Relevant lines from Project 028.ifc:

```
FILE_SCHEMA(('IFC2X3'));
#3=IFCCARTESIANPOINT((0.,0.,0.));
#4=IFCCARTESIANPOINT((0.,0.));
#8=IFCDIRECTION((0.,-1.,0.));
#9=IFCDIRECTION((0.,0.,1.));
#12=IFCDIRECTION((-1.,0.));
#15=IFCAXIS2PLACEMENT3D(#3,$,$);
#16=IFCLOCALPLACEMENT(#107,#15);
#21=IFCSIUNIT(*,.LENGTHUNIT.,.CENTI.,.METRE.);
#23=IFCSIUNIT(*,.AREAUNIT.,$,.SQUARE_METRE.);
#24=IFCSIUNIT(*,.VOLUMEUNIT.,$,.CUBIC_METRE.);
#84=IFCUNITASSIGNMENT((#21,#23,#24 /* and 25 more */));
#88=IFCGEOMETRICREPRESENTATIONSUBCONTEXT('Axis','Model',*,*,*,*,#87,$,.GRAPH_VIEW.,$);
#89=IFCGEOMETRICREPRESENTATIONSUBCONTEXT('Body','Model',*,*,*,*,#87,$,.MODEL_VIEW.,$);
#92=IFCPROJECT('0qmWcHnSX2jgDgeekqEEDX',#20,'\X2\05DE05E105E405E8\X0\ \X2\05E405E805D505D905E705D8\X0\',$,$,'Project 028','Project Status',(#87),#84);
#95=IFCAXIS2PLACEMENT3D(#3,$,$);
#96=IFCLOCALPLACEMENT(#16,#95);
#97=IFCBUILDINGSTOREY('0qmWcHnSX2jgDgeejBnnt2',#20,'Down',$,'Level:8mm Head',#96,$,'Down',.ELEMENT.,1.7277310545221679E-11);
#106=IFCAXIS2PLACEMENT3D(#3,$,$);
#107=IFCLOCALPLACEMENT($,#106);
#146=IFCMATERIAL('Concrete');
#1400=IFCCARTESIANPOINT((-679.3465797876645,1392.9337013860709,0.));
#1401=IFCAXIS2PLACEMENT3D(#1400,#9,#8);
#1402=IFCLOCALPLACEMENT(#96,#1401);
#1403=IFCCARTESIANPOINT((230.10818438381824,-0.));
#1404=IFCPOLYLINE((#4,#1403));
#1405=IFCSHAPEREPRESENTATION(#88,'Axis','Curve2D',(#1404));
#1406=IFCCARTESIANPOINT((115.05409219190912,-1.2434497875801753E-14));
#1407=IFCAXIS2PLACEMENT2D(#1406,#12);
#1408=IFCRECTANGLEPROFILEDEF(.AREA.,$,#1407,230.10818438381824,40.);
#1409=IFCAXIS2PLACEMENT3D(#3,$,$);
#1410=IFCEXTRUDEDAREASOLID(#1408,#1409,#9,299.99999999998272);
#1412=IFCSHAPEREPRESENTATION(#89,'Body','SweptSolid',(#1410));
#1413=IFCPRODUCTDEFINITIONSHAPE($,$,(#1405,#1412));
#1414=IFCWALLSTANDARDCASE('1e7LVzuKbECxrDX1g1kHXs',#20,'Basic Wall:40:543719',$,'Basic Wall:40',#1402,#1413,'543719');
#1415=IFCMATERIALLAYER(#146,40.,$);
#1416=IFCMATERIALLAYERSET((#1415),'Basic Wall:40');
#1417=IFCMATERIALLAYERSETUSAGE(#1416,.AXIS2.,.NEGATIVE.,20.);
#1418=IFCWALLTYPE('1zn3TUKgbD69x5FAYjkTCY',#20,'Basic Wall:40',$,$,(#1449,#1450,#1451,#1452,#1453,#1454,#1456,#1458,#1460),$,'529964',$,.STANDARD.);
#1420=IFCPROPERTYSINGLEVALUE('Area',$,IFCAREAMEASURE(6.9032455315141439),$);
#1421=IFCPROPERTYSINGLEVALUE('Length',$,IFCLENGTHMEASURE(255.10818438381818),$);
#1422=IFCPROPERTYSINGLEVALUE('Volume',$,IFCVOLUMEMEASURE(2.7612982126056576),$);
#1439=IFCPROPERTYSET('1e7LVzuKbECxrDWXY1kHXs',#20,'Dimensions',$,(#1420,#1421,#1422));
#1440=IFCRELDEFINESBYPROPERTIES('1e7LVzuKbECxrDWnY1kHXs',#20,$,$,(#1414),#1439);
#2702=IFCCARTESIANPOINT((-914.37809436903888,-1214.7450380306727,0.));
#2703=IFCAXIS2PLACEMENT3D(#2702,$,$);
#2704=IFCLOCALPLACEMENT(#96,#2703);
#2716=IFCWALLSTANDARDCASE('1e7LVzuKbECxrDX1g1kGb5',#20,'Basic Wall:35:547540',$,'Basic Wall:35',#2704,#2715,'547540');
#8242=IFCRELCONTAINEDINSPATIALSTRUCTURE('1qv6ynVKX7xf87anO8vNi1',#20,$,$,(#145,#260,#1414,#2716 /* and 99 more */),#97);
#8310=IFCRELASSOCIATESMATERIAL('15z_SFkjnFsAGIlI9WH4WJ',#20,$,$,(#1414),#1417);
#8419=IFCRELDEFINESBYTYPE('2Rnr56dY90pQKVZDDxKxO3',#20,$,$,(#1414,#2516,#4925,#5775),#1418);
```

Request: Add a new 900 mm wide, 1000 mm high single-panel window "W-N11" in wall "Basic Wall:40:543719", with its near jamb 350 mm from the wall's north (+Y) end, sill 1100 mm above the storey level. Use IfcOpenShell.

```python
import numpy as np
import ifcopenshell
import ifcopenshell.api.feature
import ifcopenshell.api.geometry
import ifcopenshell.api.pset
import ifcopenshell.api.root
import ifcopenshell.api.spatial
import ifcopenshell.api.type
import ifcopenshell.geom
import ifcopenshell.util.element
import ifcopenshell.util.placement
import ifcopenshell.util.representation
import ifcopenshell.util.shape
import ifcopenshell.util.unit

model = ifcopenshell.open("Project 028.ifc")
unit_scale = ifcopenshell.util.unit.calculate_unit_scale(model)
area_scale = ifcopenshell.util.unit.calculate_unit_scale(model, "AREAUNIT")
volume_scale = ifcopenshell.util.unit.calculate_unit_scale(model, "VOLUMEUNIT")
settings = ifcopenshell.geom.settings()


def volume(element):
    """Net volume in cubic metres, openings subtracted."""
    shape = ifcopenshell.geom.create_shape(settings, element)
    return ifcopenshell.util.shape.get_volume(shape.geometry)


wall = model.by_id(1414)
storey = ifcopenshell.util.element.get_container(wall, ifc_class="IfcBuildingStorey")
context = ifcopenshell.util.representation.get_context(model, "Model", "Body", "MODEL_VIEW")
before = volume(wall)

width, height, from_end, sill = 0.9, 1, 0.35, 1.1  # metres

# The wall runs along its own X axis, and the end named is its -X end.
wall_shape = ifcopenshell.geom.create_shape(settings, wall)
x, y, z = ifcopenshell.util.shape.get_vertices(wall_shape.geometry).T
start = x.min() + from_end
face, thickness = float(y.min()), float(y.max() - y.min())
wall_matrix = ifcopenshell.util.placement.get_local_placement(wall.ObjectPlacement)
level = ifcopenshell.util.placement.get_local_placement(storey.ObjectPlacement)[2, 3]


def in_wall(x, y):
    """Placement at x, y metres in the wall's axes, at sill height."""
    matrix = wall_matrix.copy()
    matrix[:, 3] = wall_matrix @ np.array([x / unit_scale, y / unit_scale, 0.0, 1.0])
    matrix[2, 3] = level + sill / unit_scale
    return matrix


# Opening: a box that overshoots both wall faces by 50 mm.
opening = ifcopenshell.api.root.create_entity(model, ifc_class="IfcOpeningElement")
box = ifcopenshell.api.geometry.add_wall_representation(
    model, context=context, length=width, height=height, thickness=thickness + 0.1
)
ifcopenshell.api.geometry.assign_representation(model, product=opening, representation=box)
ifcopenshell.api.geometry.edit_object_placement(model, product=opening, matrix=in_wall(start, face - 0.05), is_si=False)
ifcopenshell.api.feature.add_feature(model, feature=opening, element=wall)

window = ifcopenshell.api.root.create_entity(model, ifc_class="IfcWindow", name="W-N11")
window.OverallWidth, window.OverallHeight = width / unit_scale, height / unit_scale
body = ifcopenshell.api.geometry.add_window_representation(
    model,
    context=context,
    overall_width=window.OverallWidth,
    overall_height=window.OverallHeight,
    partition_type="SINGLE_PANEL",
)
ifcopenshell.api.geometry.assign_representation(model, product=window, representation=body)
ifcopenshell.api.spatial.assign_container(model, products=[window], relating_structure=storey)
fills = ifcopenshell.api.feature.add_filling(model, opening=opening, element=window)
fills.OwnerHistory = window.OwnerHistory  # required in IFC2X3

# IFC2X3 keeps the operation on the window style.
style = ifcopenshell.api.root.create_entity(model, ifc_class="IfcWindowStyle", name="W-N11")
style.OperationType, style.ConstructionType = "SINGLE_PANEL", "NOTDEFINED"
style.ParameterTakesPrecedence = style.Sizeable = False
ifcopenshell.api.type.assign_type(model, related_objects=[window], relating_type=style)

# Centre the window in the wall's thickness.
ifcopenshell.api.geometry.edit_object_placement(model, product=window, matrix=in_wall(start, face), is_si=False)
window_shape = ifcopenshell.geom.create_shape(settings, window)
depth = ifcopenshell.util.shape.get_vertices(window_shape.geometry)[:, 1]
offset = face + thickness / 2 - (depth.min() + depth.max()) / 2
ifcopenshell.api.geometry.edit_object_placement(model, product=window, matrix=in_wall(start, offset), is_si=False)

after = volume(wall)

# Update the wall's stored quantities.
pset = model.by_id(ifcopenshell.util.element.get_pset(wall, "Dimensions", should_inherit=False)["id"])
ifcopenshell.api.pset.edit_pset(model, pset=pset, properties={
    "Area": model.create_entity("IfcAreaMeasure", after / thickness / area_scale),
    "Volume": model.create_entity("IfcVolumeMeasure", after / volume_scale),
})

print(f"wall volume {before:.3f} -> {after:.3f} m3")

model.write("Project 028_v2.ifc")
```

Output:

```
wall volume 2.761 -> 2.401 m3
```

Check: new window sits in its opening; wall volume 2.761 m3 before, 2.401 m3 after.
